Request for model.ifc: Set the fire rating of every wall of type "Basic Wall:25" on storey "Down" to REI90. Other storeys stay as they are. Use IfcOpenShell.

First a look at what the model holds.

```python
import ifcopenshell
import ifcopenshell.util.element

model = ifcopenshell.open("model.ifc")
print(model.schema)
storey = next(s for s in model.by_type("IfcBuildingStorey") if s.Name == "Down")
walls = [e for e in ifcopenshell.util.element.get_decomposition(storey) if e.is_a("IfcWall")]
seen = {}
for e in walls:
    element_type = ifcopenshell.util.element.get_type(e)
    key = (element_type.Name if element_type != e and element_type else None, ifcopenshell.util.element.get_pset(e, "Pset_WallCommon", "FireRating"))
    seen[key] = seen.get(key, 0) + 1
for (name, value), count in sorted(seen.items(), key=str):
    print(count, "x", name, "|", value)
```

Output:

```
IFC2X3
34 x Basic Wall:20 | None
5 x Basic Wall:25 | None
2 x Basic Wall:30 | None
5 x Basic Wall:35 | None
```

```python
import ifcopenshell
import ifcopenshell.api.pset
import ifcopenshell.util.element

model = ifcopenshell.open("model.ifc")

storey = next(s for s in model.by_type("IfcBuildingStorey") if s.Name == "Down")
walls = [e for e in ifcopenshell.util.element.get_decomposition(storey) if e.is_a("IfcWall")]

count = 0
for e in walls:
    element_type = ifcopenshell.util.element.get_type(e)
    if element_type in (None, e) or element_type.Name != "Basic Wall:25":
        continue
    # add_pset returns the element's existing set when there is one.
    pset = ifcopenshell.api.pset.add_pset(model, product=e, name="Pset_WallCommon")
    ifcopenshell.api.pset.edit_pset(model, pset=pset, properties={"FireRating": "REI90"})
    count += 1

print(count, "walls updated")

model.write("model_rev.ifc")
```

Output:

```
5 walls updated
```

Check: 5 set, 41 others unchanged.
